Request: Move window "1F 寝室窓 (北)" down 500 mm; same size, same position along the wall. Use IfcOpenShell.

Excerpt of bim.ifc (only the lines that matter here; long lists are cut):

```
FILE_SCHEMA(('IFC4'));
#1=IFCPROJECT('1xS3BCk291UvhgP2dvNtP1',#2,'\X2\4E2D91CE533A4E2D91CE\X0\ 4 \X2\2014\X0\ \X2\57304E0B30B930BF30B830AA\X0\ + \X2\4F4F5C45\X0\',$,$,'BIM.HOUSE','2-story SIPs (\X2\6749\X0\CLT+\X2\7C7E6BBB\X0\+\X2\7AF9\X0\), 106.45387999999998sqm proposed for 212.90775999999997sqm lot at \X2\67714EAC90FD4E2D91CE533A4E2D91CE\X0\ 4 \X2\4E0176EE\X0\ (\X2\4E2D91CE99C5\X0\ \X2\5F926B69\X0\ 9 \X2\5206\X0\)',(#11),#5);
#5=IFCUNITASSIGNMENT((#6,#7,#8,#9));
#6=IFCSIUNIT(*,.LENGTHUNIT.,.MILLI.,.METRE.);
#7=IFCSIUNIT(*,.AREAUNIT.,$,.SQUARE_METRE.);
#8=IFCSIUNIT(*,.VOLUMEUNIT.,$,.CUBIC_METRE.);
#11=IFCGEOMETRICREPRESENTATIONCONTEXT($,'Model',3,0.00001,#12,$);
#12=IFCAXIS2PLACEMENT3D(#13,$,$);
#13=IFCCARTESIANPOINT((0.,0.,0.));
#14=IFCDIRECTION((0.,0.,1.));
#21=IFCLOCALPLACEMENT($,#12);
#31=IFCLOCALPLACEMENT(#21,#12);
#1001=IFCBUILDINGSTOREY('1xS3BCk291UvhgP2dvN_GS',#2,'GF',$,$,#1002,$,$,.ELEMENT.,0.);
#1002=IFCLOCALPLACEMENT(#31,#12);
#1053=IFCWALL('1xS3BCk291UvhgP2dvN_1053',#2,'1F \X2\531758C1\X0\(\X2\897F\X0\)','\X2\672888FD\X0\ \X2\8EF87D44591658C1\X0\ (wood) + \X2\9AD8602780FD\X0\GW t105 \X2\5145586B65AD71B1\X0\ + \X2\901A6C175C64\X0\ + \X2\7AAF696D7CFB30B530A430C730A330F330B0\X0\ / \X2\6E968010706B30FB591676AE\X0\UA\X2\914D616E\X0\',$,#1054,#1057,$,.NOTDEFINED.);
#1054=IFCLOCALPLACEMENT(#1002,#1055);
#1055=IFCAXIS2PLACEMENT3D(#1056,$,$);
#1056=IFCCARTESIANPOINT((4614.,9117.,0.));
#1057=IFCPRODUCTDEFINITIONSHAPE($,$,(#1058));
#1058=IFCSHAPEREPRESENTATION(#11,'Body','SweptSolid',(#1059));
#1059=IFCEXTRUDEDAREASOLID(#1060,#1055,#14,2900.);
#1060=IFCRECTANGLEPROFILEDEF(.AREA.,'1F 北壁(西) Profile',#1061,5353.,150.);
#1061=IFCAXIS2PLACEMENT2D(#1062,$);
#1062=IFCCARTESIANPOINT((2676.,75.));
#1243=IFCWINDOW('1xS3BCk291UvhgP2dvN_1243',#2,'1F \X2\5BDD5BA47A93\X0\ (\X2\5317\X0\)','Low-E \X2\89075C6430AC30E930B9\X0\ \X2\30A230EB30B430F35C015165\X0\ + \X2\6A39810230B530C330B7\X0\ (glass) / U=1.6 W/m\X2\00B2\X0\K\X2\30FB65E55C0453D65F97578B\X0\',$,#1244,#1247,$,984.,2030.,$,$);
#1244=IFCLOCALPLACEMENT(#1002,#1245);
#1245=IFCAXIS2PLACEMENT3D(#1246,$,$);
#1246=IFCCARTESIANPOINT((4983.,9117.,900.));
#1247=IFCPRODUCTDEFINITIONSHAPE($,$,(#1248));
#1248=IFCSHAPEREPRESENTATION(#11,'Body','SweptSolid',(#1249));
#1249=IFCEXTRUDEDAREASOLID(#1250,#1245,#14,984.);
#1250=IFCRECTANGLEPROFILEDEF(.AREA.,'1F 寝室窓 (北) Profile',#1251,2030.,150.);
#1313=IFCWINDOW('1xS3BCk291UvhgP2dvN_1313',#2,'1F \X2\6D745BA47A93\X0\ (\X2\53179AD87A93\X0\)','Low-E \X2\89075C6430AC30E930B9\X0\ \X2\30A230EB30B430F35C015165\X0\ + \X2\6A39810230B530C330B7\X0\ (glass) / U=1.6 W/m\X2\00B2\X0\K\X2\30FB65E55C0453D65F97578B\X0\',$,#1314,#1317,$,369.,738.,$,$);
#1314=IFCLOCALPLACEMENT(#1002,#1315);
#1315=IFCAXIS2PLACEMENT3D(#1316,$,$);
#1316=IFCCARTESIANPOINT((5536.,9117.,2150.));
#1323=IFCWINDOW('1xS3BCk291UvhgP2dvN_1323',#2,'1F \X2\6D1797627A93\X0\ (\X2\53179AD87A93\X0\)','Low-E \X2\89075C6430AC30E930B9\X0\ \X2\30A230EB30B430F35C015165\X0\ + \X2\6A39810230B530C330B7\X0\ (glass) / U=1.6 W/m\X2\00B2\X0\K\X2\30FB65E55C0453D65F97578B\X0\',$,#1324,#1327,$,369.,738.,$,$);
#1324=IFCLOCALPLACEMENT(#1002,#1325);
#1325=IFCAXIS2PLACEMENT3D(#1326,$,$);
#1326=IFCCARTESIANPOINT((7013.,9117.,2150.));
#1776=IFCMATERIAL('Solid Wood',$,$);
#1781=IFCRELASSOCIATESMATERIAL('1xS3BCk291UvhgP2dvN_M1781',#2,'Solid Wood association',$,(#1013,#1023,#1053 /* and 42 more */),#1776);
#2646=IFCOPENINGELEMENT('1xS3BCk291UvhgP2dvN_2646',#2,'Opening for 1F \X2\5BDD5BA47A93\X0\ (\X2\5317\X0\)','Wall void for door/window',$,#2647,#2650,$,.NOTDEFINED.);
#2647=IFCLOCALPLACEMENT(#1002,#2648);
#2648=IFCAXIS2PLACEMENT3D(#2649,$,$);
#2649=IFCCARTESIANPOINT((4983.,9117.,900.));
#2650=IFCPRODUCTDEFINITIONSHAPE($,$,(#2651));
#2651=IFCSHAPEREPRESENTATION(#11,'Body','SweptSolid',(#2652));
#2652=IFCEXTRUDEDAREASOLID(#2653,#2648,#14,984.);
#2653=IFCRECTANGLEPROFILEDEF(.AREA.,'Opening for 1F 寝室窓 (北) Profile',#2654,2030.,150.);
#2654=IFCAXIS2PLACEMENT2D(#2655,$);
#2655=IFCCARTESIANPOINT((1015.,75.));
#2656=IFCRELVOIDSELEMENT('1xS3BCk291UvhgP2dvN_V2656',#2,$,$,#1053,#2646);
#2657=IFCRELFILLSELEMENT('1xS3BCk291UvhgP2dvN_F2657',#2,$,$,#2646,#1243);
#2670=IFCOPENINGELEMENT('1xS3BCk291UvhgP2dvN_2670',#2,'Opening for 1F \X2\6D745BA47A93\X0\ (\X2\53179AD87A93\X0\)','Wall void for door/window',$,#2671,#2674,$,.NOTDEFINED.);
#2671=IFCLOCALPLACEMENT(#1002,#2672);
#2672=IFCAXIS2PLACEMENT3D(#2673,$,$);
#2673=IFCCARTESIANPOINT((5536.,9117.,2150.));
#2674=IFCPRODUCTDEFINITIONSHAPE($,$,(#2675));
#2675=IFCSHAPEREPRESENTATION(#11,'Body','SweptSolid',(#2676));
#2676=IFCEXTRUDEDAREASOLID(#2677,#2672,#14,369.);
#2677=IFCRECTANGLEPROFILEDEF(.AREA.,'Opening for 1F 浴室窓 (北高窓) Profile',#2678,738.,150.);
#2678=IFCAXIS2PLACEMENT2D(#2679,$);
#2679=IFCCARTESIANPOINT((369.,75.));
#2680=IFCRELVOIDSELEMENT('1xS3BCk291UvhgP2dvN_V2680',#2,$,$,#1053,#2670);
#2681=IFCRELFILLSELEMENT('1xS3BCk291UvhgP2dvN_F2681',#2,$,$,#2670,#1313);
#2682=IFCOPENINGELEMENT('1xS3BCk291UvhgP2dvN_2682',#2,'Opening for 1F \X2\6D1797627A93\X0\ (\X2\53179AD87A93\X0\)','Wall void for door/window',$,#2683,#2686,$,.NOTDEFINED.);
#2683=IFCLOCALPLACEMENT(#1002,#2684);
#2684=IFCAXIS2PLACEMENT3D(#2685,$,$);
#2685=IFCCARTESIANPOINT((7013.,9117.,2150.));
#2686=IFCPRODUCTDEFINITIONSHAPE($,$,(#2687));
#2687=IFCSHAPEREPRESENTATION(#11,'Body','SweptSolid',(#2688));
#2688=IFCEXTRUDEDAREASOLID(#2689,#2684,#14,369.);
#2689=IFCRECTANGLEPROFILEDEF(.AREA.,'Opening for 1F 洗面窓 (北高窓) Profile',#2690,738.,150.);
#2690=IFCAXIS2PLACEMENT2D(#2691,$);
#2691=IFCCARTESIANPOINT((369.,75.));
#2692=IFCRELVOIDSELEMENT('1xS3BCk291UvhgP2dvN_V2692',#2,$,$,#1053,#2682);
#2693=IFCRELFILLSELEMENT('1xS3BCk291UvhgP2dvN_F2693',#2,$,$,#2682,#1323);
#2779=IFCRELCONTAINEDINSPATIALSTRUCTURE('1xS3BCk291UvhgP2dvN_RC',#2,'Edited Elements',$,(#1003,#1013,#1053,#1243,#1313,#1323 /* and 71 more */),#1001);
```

```python
import numpy as np
import ifcopenshell
import ifcopenshell.api.geometry
import ifcopenshell.util.placement
import ifcopenshell.util.unit

model = ifcopenshell.open("bim.ifc")
unit_scale = ifcopenshell.util.unit.calculate_unit_scale(model)

window = model.by_guid("1xS3BCk291UvhgP2dvN_1243")
opening = window.FillsVoids[0].RelatingOpeningElement
dz = -0.5 / unit_scale

shift = np.array([0.0, 0.0, dz])
# The window is not placed relative to its opening, so move both.
for product in (opening, window):
    matrix = ifcopenshell.util.placement.get_local_placement(product.ObjectPlacement)
    matrix[:3, 3] += shift
    ifcopenshell.api.geometry.edit_object_placement(model, product=product, matrix=matrix, is_si=False)

print(f"moved by {dz * unit_scale:+.3f} m")

model.write("bim_edited.ifc")
```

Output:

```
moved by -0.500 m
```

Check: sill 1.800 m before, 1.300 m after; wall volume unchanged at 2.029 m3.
